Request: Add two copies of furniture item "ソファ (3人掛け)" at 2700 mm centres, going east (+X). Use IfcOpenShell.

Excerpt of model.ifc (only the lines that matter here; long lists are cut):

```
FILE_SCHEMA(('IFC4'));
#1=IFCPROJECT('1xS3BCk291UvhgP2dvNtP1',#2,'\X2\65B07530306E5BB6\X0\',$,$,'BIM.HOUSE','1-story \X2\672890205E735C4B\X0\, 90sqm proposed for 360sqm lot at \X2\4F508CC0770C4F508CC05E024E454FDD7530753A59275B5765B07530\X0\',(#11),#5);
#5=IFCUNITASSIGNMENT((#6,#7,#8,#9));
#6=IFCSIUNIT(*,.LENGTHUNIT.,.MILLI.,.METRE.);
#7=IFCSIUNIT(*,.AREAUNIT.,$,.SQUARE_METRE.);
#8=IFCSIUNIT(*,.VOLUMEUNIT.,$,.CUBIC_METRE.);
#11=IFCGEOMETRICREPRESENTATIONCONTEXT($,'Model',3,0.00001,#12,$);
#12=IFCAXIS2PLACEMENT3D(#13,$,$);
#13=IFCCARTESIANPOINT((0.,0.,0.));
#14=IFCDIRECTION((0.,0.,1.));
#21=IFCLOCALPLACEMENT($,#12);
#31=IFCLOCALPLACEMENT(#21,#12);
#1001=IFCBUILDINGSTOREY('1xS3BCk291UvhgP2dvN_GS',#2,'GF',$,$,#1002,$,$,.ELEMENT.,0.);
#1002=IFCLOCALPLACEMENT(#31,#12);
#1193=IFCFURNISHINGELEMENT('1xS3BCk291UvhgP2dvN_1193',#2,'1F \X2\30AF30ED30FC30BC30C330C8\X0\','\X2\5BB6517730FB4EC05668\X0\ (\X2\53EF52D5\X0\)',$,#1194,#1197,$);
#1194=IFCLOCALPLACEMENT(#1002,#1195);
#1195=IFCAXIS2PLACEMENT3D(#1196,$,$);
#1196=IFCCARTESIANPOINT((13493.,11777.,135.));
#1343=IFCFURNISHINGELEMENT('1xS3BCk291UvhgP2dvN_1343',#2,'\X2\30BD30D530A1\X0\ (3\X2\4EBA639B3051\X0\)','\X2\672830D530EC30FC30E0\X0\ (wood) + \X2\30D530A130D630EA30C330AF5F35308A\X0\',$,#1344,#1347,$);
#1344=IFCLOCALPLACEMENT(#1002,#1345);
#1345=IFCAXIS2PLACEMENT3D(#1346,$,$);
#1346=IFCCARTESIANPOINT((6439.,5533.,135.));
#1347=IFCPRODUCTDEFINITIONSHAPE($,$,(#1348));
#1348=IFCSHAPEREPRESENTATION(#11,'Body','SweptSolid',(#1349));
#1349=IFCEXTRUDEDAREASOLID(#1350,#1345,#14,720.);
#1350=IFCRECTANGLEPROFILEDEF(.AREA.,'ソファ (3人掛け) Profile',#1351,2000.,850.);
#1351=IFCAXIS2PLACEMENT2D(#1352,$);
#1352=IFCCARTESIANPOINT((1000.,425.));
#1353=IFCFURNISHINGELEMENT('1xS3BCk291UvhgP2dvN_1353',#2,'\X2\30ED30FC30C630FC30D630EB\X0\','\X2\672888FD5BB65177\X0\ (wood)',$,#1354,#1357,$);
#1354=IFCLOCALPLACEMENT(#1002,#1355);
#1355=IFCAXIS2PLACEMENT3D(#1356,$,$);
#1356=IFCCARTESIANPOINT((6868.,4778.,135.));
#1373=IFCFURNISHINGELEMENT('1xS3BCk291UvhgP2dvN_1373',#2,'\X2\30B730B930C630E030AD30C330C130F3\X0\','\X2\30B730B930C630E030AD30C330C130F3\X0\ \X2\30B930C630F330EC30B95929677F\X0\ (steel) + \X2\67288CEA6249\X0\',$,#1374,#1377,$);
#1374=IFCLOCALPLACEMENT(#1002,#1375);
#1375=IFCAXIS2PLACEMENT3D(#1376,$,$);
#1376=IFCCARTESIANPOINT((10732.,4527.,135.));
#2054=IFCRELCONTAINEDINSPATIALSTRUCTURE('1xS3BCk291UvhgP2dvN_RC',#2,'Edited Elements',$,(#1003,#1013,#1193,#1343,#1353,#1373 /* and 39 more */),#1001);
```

```python
import numpy as np
import ifcopenshell
import ifcopenshell.api.geometry
import ifcopenshell.api.root
import ifcopenshell.util.element
import ifcopenshell.util.placement
import ifcopenshell.util.unit

model = ifcopenshell.open("model.ifc")
unit_scale = ifcopenshell.util.unit.calculate_unit_scale(model)


def reuse_history(source, copy):
    """copy_class also copies each property set's owner history, people and application; keep the originals."""
    for rel in copy.IsDefinedBy:
        if rel.is_a("IfcRelDefinesByProperties") and (history := rel.RelatingPropertyDefinition.OwnerHistory):
            rel.RelatingPropertyDefinition.OwnerHistory = source.OwnerHistory
            ifcopenshell.util.element.remove_deep2(model, history)


source = model.by_guid("1xS3BCk291UvhgP2dvN_1343")
base = ifcopenshell.util.placement.get_local_placement(source.ObjectPlacement)
step = np.array([1.0, 0.0, 0.0]) * 2.7 / unit_scale

for i in range(1, 3):
    copy = ifcopenshell.api.root.copy_class(model, product=source)
    copy.Representation = ifcopenshell.util.element.copy_deep(
        model, source.Representation, exclude=["IfcGeometricRepresentationContext", "IfcRepresentationMap"]
    )
    reuse_history(source, copy)
    matrix = base.copy()
    matrix[:3, 3] += i * step
    print("added at", matrix[:3, 3].round(3) + 0.0)
    ifcopenshell.api.geometry.edit_object_placement(model, product=copy, matrix=matrix, is_si=False)

model.write("model_edited.ifc")
```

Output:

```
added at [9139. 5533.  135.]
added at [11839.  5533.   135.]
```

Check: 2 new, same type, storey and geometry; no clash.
